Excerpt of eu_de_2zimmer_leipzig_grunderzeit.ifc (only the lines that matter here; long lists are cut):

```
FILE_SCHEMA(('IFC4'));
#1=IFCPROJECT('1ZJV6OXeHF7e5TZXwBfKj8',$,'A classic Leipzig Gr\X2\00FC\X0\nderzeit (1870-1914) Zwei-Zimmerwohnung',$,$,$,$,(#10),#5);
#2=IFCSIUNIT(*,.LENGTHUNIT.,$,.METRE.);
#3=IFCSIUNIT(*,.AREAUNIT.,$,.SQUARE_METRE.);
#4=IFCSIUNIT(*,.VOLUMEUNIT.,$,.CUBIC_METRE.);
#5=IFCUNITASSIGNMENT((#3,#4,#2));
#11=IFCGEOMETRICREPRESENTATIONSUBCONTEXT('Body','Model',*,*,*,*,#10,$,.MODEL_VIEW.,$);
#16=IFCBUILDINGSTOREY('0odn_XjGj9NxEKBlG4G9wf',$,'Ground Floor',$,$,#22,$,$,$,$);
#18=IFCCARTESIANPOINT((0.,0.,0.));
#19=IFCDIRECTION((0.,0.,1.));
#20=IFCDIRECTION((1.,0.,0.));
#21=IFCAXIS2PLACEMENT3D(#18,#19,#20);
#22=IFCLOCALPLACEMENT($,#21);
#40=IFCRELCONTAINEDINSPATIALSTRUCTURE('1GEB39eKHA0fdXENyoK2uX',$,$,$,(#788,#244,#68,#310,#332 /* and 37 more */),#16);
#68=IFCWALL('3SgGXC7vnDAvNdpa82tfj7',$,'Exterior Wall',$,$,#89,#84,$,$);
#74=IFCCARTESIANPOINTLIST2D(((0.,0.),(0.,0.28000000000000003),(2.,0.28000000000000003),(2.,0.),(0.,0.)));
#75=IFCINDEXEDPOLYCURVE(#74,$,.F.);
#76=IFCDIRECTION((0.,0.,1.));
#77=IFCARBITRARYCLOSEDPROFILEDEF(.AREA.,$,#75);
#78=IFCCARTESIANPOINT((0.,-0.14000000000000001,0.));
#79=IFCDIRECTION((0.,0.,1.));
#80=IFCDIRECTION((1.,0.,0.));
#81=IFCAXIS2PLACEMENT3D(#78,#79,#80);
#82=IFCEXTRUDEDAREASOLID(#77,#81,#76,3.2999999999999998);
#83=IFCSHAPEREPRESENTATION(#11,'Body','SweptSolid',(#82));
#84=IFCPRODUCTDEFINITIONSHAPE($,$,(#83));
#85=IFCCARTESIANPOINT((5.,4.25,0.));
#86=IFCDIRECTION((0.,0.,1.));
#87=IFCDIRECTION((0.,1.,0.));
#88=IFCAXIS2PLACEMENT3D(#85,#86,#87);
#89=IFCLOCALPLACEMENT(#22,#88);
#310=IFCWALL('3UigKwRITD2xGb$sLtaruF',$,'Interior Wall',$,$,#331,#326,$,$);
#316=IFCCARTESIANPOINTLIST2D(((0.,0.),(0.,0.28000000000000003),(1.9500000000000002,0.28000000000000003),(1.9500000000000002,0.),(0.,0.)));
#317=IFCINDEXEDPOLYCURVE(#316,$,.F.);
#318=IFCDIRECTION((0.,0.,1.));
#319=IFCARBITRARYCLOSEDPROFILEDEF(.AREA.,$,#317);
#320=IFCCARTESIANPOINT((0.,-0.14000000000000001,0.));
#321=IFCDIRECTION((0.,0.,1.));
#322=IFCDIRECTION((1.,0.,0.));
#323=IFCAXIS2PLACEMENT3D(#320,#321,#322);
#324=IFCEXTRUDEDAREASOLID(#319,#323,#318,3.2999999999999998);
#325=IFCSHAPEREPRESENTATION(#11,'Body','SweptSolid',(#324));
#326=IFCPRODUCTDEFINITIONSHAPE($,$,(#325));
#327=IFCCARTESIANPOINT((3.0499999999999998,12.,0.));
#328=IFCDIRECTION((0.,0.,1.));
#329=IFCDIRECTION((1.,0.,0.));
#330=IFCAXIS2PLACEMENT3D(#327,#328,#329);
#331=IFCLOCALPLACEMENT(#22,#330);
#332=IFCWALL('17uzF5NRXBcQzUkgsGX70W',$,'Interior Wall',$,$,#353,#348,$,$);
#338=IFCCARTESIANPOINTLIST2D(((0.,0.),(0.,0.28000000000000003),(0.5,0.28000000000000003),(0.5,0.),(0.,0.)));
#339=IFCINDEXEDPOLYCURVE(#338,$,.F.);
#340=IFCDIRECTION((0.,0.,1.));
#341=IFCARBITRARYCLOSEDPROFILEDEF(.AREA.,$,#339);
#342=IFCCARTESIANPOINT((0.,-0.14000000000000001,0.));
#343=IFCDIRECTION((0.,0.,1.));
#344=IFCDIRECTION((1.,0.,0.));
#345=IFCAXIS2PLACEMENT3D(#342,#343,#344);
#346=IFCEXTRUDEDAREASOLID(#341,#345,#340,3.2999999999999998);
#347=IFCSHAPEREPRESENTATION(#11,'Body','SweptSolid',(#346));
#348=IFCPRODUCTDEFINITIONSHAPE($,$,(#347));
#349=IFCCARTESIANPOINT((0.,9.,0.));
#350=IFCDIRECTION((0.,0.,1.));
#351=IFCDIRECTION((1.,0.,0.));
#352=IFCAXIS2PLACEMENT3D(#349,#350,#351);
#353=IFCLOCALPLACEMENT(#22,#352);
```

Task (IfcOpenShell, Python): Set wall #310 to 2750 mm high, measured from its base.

```python
import ifcopenshell
import ifcopenshell.geom
import ifcopenshell.util.representation
import ifcopenshell.util.shape
import ifcopenshell.util.unit

model = ifcopenshell.open("eu_de_2zimmer_leipzig_grunderzeit.ifc")
unit_scale = ifcopenshell.util.unit.calculate_unit_scale(model)
settings = ifcopenshell.geom.settings()


def volume(element):
    """Net volume in cubic metres, openings subtracted."""
    shape = ifcopenshell.geom.create_shape(settings, element)
    return ifcopenshell.util.shape.get_volume(shape.geometry)


wall = model.by_guid("3UigKwRITD2xGb$sLtaruF")
before = volume(wall)

body = ifcopenshell.util.representation.get_representation(wall, "Model", "Body")
solid = body.Items[0]
old_height = solid.Depth
solid.Depth = 2.75 / unit_scale
after = volume(wall)

print(f"height {old_height:g} -> {solid.Depth:g}, volume {before:.3f} -> {after:.3f} m3")

model.write("eu_de_2zimmer_leipzig_grunderzeit_edited.ifc")
```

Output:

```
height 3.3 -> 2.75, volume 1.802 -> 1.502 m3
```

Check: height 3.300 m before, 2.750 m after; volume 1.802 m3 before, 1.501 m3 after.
